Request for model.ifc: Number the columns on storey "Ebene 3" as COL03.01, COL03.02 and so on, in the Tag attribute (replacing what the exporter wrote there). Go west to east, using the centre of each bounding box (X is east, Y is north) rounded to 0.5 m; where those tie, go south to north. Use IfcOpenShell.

First a look at what the model holds.

```python
import ifcopenshell
import ifcopenshell.util.element
import ifcopenshell.util.placement

model = ifcopenshell.open("model.ifc")
print(model.schema)
storey = next(s for s in model.by_type("IfcBuildingStorey") if s.Name == "Ebene 3")
columns = [e for e in ifcopenshell.util.element.get_decomposition(storey) if e.is_a("IfcColumn")]
for e in sorted(columns, key=lambda e: e.id()):
    origin = ifcopenshell.util.placement.get_local_placement(e.ObjectPlacement)[:3, 3]
    print(e.id(), e.Tag, e.Name, origin.round(2) + 0.0, sep=" | ")
```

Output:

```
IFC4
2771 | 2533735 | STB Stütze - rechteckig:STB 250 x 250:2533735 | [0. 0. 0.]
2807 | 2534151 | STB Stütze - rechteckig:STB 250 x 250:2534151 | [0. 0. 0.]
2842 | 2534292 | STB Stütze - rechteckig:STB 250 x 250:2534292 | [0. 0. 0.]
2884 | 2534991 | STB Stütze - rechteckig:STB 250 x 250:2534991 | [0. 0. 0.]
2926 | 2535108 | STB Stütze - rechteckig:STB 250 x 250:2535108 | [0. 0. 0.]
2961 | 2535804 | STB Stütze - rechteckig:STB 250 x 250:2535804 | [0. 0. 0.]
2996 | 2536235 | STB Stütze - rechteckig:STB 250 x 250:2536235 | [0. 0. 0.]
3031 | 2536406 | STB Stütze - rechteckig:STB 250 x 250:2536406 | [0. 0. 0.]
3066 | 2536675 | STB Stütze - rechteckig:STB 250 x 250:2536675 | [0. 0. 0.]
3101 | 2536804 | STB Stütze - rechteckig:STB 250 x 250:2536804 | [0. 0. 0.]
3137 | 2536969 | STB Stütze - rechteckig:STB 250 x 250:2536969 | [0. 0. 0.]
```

```python
import ifcopenshell
import ifcopenshell.geom
import ifcopenshell.util.element
import ifcopenshell.util.shape

model = ifcopenshell.open("model.ifc")
settings = ifcopenshell.geom.settings()
settings.set("use-world-coords", True)


def centre(element):
    shape = ifcopenshell.geom.create_shape(settings, element)
    return ifcopenshell.util.shape.get_bbox_centroid(shape.geometry)


storey = next(s for s in model.by_type("IfcBuildingStorey") if s.Name == "Ebene 3")
columns = [e for e in ifcopenshell.util.element.get_decomposition(storey) if e.is_a("IfcColumn")]

# Insertion points can sit at a corner or the storey origin, so sort by the geometry (in metres).
centres = {e: centre(e) for e in columns}
columns.sort(key=lambda e: (round(centres[e][0] / 0.5), centres[e][1]))

for i, e in enumerate(columns, start=1):
    number = f"COL03.{i:02d}"
    e.Tag = number
    print(e.id(), number)

model.write("model-out.ifc")
```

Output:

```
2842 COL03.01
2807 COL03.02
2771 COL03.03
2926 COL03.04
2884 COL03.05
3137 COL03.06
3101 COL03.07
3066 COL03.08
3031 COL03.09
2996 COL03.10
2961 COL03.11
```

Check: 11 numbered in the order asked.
